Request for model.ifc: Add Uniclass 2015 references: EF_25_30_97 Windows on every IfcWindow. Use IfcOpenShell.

First a look at what the model holds.

```python
import ifcopenshell

model = ifcopenshell.open("model.ifc")
print(model.schema)
print("classifications:", [c.Name for c in model.by_type("IfcClassification")])
for ifc_class in ("IfcDoor", "IfcRoof", "IfcStair", "IfcWall", "IfcWindow"):
    print(ifc_class, len(model.by_type(ifc_class)))
```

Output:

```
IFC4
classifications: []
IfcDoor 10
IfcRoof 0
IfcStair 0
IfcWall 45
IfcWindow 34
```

```python
import ifcopenshell
import ifcopenshell.api.classification

model = ifcopenshell.open("model.ifc")

system = ifcopenshell.api.classification.add_classification(model, classification="Uniclass 2015")

codes = {
    "IfcWindow": ("EF_25_30_97", "Windows"),
}
for ifc_class, (code, name) in codes.items():
    products = model.by_type(ifc_class)
    ifcopenshell.api.classification.add_reference(
        model, products=products, classification=system, identification=code, name=name
    )
    print(code, len(products))

model.write("model_updated.ifc")
```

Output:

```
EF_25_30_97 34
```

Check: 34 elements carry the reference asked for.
